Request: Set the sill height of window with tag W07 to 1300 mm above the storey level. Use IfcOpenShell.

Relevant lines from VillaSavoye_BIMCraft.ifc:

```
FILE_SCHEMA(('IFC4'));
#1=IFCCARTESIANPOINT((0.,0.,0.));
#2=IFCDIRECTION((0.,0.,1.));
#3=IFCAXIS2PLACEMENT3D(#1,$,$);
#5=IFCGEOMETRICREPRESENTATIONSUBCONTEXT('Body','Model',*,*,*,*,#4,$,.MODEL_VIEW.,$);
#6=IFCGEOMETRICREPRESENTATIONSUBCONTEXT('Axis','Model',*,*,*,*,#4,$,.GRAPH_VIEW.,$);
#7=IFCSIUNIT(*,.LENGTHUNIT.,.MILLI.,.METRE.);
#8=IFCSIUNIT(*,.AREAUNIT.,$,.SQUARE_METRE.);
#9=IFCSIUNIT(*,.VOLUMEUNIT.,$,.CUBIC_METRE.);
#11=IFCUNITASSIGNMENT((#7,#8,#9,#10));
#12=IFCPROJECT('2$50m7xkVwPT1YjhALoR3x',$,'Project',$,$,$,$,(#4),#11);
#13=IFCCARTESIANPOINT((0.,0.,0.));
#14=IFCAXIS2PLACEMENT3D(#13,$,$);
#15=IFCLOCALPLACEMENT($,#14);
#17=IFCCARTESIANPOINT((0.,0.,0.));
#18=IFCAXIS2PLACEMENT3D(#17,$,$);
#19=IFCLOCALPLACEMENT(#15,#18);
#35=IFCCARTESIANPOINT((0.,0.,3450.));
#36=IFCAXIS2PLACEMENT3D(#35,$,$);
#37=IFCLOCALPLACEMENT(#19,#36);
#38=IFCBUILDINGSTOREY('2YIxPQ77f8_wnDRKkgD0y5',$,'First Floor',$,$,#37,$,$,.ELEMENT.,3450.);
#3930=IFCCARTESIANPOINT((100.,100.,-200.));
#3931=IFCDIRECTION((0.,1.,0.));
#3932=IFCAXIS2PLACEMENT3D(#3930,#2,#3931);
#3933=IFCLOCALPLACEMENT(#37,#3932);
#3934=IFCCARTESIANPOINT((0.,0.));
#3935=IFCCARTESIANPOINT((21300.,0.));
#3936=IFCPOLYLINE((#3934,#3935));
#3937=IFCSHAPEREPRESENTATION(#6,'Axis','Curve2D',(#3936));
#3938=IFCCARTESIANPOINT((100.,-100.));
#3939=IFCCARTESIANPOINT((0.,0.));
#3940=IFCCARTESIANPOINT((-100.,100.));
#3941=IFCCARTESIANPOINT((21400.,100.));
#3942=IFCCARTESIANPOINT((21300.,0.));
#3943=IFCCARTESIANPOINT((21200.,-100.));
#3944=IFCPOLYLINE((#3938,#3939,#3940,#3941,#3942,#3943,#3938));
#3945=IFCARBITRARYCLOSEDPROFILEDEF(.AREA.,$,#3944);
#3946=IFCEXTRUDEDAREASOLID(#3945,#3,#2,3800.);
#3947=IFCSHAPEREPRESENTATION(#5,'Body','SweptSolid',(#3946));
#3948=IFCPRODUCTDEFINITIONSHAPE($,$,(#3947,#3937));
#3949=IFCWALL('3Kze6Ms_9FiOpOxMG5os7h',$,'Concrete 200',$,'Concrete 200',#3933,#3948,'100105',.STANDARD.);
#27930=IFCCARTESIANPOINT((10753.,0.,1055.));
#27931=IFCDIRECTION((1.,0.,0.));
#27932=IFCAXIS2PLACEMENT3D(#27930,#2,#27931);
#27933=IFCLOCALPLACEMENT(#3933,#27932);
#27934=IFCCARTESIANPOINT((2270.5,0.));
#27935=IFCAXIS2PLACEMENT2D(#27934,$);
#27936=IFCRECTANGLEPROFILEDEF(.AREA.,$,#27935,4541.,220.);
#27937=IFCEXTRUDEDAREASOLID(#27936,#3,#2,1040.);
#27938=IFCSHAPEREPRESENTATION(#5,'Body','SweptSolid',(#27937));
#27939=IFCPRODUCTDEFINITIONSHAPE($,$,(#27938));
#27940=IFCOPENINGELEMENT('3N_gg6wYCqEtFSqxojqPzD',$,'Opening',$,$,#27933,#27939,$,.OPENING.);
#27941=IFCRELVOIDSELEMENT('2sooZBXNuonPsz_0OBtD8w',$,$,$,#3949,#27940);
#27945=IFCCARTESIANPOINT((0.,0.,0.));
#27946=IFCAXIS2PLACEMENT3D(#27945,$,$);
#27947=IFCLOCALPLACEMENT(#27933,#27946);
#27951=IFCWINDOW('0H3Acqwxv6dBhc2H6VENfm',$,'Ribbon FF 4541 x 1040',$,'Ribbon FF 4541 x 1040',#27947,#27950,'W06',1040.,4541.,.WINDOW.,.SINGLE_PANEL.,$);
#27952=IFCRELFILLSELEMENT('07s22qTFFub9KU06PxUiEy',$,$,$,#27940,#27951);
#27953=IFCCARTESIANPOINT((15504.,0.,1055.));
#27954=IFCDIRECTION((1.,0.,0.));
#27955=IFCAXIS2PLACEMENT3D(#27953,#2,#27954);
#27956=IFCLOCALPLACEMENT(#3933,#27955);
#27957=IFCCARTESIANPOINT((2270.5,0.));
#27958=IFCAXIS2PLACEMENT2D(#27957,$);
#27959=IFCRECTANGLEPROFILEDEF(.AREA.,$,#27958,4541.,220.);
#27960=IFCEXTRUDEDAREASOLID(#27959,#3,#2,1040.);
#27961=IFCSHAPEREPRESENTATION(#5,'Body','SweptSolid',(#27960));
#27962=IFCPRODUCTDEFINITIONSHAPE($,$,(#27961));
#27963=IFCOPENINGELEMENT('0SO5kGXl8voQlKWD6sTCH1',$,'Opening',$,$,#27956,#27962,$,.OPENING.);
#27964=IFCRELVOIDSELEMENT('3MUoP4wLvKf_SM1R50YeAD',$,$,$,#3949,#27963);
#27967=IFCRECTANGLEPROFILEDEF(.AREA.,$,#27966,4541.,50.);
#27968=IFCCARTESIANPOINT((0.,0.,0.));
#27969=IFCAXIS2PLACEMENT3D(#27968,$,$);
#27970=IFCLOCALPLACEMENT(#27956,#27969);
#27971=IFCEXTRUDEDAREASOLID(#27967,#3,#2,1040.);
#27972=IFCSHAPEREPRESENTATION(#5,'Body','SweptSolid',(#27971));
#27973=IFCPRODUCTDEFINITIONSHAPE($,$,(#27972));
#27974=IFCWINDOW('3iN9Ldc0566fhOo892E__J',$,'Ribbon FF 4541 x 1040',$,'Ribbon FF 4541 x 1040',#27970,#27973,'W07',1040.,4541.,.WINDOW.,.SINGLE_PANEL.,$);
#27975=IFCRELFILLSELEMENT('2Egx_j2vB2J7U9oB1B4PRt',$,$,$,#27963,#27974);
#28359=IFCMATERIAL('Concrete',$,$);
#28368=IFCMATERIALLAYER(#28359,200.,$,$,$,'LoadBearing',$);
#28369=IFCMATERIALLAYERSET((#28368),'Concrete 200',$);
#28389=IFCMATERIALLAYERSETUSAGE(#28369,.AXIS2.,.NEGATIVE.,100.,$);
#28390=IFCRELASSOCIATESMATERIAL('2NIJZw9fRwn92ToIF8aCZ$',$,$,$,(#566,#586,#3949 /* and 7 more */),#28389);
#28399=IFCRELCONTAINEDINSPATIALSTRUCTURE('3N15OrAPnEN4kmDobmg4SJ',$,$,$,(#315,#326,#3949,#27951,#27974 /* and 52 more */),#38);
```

```python
import numpy as np
import ifcopenshell
import ifcopenshell.api.geometry
import ifcopenshell.geom
import ifcopenshell.util.element
import ifcopenshell.util.placement
import ifcopenshell.util.shape
import ifcopenshell.util.unit

model = ifcopenshell.open("VillaSavoye_BIMCraft.ifc")
unit_scale = ifcopenshell.util.unit.calculate_unit_scale(model)

window = model.by_guid("3iN9Ldc0566fhOo892E__J")
opening = window.FillsVoids[0].RelatingOpeningElement
storey = ifcopenshell.util.element.get_container(window, ifc_class="IfcBuildingStorey")
level = ifcopenshell.util.placement.get_local_placement(storey.ObjectPlacement)[2, 3]

# The opening's origin need not be at the sill, so measure its lowest point.
shape = ifcopenshell.geom.create_shape(ifcopenshell.geom.settings(), opening)
bottom = ifcopenshell.util.shape.get_shape_bottom_elevation(shape, shape.geometry) / unit_scale
dz = level + 1.3 / unit_scale - bottom

shift = np.array([0.0, 0.0, dz])
# The window is placed relative to its opening, so it follows when the opening moves.
matrix = ifcopenshell.util.placement.get_local_placement(opening.ObjectPlacement)
matrix[:3, 3] += shift
ifcopenshell.api.geometry.edit_object_placement(
    model, product=opening, matrix=matrix, is_si=False, should_transform_children=True
)

print(f"moved by {dz * unit_scale:+.3f} m")

model.write("VillaSavoye_BIMCraft-out.ifc")
```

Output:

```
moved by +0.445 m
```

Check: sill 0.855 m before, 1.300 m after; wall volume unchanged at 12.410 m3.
